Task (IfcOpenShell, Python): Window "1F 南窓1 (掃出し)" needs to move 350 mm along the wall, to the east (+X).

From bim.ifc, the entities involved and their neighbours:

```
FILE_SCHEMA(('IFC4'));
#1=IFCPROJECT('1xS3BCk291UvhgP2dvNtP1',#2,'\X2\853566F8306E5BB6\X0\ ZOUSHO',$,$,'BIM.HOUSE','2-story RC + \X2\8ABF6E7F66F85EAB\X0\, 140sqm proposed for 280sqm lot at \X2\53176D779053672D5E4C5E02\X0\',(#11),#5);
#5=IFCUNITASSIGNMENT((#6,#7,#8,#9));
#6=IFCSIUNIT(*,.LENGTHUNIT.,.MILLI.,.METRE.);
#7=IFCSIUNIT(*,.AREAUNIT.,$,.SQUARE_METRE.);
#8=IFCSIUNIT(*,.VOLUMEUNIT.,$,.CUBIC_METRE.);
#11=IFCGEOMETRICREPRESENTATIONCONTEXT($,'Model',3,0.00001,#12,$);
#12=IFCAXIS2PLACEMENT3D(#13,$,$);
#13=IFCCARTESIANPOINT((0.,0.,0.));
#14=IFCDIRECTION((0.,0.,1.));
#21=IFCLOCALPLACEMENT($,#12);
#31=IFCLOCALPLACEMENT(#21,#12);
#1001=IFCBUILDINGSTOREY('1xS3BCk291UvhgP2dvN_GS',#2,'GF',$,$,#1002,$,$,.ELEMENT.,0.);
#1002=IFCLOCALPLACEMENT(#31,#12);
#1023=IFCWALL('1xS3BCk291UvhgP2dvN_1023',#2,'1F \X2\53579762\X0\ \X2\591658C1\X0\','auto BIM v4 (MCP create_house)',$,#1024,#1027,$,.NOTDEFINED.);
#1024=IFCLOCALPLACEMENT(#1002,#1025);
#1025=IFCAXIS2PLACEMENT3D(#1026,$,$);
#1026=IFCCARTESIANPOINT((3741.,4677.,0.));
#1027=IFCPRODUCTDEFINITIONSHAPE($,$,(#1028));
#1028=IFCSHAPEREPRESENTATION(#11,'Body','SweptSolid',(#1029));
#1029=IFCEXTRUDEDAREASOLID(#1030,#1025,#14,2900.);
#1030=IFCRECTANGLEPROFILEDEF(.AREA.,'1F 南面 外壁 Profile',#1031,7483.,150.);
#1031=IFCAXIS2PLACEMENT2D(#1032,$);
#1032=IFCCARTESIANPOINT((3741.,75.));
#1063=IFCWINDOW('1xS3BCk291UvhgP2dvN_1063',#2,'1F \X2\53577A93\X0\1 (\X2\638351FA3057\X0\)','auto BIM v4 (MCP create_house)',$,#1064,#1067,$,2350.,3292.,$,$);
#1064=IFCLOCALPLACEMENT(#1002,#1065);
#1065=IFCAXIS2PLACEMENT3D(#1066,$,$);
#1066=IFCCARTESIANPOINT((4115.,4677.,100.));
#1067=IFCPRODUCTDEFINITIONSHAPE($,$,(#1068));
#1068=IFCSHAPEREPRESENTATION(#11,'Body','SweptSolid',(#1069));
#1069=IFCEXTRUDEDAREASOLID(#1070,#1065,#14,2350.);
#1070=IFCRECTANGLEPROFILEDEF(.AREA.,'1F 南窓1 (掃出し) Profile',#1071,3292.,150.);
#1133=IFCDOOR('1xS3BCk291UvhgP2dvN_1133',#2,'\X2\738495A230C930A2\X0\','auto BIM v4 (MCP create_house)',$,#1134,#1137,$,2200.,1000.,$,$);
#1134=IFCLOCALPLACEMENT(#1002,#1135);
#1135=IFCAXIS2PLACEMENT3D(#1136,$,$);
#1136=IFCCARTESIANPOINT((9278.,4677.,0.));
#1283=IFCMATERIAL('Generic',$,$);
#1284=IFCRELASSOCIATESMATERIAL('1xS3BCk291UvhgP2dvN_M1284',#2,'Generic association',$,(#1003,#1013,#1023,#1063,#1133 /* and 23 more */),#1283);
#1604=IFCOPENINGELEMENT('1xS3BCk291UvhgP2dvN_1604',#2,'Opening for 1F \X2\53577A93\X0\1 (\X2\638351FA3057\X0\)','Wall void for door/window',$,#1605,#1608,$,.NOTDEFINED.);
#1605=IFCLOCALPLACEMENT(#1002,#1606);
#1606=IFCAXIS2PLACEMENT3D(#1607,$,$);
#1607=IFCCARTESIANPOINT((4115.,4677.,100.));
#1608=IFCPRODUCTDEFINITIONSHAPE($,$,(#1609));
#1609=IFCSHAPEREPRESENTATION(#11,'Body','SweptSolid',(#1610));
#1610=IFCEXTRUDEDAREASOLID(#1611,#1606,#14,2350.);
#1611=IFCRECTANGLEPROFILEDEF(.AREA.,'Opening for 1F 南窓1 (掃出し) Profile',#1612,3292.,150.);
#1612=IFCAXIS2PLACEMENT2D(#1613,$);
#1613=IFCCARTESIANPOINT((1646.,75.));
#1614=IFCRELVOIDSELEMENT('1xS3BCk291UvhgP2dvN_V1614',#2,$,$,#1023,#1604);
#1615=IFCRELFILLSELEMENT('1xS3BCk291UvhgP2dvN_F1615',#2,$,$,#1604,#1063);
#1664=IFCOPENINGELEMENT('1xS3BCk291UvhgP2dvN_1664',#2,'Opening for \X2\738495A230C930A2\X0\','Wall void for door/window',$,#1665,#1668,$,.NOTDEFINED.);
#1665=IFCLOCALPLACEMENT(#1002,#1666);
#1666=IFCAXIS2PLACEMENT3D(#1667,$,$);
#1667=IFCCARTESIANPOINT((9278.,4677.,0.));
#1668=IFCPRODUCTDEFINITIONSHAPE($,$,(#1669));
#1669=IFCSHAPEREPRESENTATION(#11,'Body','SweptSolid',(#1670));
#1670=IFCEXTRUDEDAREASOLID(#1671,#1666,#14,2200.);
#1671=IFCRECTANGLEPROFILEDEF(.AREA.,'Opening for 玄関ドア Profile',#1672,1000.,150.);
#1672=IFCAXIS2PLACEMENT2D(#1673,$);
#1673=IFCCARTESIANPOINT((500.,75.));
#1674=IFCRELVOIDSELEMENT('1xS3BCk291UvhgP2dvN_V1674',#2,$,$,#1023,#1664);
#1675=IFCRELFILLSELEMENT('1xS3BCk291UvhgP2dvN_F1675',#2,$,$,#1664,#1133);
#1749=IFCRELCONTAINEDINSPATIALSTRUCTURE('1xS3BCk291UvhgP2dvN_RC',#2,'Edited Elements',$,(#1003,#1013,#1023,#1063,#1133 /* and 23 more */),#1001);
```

```python
import ifcopenshell
import ifcopenshell.api.geometry
import ifcopenshell.util.placement
import ifcopenshell.util.unit

model = ifcopenshell.open("bim.ifc")
unit_scale = ifcopenshell.util.unit.calculate_unit_scale(model)

window = model.by_id(1063)
opening = window.FillsVoids[0].RelatingOpeningElement
wall = opening.VoidsElements[0].RelatingBuildingElement

wall_matrix = ifcopenshell.util.placement.get_local_placement(wall.ObjectPlacement)
shift = wall_matrix[:3, 0] * 0.35 / unit_scale
before = ifcopenshell.util.placement.get_local_placement(window.ObjectPlacement)[:3, 3].copy()

# The window is not placed relative to its opening, so move both.
for product in (opening, window):
    matrix = ifcopenshell.util.placement.get_local_placement(product.ObjectPlacement)
    matrix[:3, 3] += shift
    ifcopenshell.api.geometry.edit_object_placement(model, product=product, matrix=matrix, is_si=False)

after = ifcopenshell.util.placement.get_local_placement(window.ObjectPlacement)[:3, 3]
print("window moved by", (after - before).round(3) + 0.0)

model.write("bim_edited.ifc")
```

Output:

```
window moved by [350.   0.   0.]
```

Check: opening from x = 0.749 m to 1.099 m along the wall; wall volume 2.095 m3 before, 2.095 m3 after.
